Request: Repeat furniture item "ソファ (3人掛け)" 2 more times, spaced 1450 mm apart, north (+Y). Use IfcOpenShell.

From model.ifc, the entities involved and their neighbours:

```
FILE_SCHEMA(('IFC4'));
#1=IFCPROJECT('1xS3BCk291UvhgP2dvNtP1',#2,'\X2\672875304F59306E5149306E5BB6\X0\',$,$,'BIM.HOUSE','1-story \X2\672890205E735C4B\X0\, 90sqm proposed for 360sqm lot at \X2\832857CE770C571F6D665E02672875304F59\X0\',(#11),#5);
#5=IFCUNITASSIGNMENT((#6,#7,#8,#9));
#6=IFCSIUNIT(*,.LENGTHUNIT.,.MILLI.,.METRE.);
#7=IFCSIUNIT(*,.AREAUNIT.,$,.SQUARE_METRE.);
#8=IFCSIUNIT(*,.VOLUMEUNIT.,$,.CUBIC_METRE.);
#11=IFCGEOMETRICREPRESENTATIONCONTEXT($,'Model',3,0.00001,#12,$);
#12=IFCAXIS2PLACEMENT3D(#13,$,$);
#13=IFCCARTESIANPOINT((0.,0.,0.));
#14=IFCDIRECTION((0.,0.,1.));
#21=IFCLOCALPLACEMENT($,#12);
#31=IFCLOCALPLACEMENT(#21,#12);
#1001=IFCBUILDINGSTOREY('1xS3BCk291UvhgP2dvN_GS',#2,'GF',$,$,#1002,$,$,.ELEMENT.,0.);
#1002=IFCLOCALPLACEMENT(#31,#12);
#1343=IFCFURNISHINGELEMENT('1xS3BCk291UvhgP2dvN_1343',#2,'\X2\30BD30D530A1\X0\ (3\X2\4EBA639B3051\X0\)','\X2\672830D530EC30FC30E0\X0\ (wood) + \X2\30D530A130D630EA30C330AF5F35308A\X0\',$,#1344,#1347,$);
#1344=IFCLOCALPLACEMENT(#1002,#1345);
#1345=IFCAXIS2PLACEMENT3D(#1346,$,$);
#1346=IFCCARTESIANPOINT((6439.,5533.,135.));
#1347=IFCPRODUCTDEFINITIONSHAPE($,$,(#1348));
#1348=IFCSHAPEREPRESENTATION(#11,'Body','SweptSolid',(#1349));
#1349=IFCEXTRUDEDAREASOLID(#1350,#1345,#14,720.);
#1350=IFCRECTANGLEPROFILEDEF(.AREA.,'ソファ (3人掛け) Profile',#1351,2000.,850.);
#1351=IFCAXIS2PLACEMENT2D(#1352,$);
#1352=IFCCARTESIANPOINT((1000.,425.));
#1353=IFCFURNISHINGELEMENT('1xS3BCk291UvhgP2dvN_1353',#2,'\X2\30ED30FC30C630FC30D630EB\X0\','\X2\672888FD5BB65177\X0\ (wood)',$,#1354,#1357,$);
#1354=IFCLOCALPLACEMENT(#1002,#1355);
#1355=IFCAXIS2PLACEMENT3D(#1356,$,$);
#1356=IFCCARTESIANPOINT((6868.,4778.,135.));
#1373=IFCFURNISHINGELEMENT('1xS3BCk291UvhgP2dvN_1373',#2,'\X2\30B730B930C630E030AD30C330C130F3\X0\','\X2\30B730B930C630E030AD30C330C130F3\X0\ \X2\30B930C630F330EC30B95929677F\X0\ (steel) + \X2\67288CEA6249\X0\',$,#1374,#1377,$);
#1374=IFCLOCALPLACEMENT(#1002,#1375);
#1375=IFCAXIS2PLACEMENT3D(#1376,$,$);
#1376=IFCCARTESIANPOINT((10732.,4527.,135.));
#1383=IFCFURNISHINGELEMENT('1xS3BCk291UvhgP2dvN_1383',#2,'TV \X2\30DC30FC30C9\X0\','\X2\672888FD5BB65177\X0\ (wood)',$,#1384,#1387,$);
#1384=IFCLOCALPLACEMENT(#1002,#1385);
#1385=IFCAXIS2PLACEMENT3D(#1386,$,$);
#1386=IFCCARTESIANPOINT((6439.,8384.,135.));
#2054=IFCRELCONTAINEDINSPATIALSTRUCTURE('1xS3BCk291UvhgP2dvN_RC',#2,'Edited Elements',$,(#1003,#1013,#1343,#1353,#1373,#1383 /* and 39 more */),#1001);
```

```python
import numpy as np
import ifcopenshell
import ifcopenshell.api.geometry
import ifcopenshell.api.root
import ifcopenshell.util.element
import ifcopenshell.util.placement

model = ifcopenshell.open("model.ifc")


def reuse_history(source, copy):
    """copy_class also copies each property set's owner history, people and application; keep the originals."""
    for rel in copy.IsDefinedBy:
        if rel.is_a("IfcRelDefinesByProperties") and (history := rel.RelatingPropertyDefinition.OwnerHistory):
            rel.RelatingPropertyDefinition.OwnerHistory = source.OwnerHistory
            ifcopenshell.util.element.remove_deep2(model, history)


source = model.by_id(1343)
base = ifcopenshell.util.placement.get_local_placement(source.ObjectPlacement)
step = np.array([0.0, 1.0, 0.0]) * 1450.0

for i in range(1, 3):
    copy = ifcopenshell.api.root.copy_class(model, product=source)
    copy.Representation = ifcopenshell.util.element.copy_deep(
        model, source.Representation, exclude=["IfcGeometricRepresentationContext", "IfcRepresentationMap"]
    )
    reuse_history(source, copy)
    matrix = base.copy()
    matrix[:3, 3] += i * step
    print("added at", matrix[:3, 3].round(3) + 0.0)
    ifcopenshell.api.geometry.edit_object_placement(model, product=copy, matrix=matrix, is_si=False)

model.write("model_rev.ifc")
```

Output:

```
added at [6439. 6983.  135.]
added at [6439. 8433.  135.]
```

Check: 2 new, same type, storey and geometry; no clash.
